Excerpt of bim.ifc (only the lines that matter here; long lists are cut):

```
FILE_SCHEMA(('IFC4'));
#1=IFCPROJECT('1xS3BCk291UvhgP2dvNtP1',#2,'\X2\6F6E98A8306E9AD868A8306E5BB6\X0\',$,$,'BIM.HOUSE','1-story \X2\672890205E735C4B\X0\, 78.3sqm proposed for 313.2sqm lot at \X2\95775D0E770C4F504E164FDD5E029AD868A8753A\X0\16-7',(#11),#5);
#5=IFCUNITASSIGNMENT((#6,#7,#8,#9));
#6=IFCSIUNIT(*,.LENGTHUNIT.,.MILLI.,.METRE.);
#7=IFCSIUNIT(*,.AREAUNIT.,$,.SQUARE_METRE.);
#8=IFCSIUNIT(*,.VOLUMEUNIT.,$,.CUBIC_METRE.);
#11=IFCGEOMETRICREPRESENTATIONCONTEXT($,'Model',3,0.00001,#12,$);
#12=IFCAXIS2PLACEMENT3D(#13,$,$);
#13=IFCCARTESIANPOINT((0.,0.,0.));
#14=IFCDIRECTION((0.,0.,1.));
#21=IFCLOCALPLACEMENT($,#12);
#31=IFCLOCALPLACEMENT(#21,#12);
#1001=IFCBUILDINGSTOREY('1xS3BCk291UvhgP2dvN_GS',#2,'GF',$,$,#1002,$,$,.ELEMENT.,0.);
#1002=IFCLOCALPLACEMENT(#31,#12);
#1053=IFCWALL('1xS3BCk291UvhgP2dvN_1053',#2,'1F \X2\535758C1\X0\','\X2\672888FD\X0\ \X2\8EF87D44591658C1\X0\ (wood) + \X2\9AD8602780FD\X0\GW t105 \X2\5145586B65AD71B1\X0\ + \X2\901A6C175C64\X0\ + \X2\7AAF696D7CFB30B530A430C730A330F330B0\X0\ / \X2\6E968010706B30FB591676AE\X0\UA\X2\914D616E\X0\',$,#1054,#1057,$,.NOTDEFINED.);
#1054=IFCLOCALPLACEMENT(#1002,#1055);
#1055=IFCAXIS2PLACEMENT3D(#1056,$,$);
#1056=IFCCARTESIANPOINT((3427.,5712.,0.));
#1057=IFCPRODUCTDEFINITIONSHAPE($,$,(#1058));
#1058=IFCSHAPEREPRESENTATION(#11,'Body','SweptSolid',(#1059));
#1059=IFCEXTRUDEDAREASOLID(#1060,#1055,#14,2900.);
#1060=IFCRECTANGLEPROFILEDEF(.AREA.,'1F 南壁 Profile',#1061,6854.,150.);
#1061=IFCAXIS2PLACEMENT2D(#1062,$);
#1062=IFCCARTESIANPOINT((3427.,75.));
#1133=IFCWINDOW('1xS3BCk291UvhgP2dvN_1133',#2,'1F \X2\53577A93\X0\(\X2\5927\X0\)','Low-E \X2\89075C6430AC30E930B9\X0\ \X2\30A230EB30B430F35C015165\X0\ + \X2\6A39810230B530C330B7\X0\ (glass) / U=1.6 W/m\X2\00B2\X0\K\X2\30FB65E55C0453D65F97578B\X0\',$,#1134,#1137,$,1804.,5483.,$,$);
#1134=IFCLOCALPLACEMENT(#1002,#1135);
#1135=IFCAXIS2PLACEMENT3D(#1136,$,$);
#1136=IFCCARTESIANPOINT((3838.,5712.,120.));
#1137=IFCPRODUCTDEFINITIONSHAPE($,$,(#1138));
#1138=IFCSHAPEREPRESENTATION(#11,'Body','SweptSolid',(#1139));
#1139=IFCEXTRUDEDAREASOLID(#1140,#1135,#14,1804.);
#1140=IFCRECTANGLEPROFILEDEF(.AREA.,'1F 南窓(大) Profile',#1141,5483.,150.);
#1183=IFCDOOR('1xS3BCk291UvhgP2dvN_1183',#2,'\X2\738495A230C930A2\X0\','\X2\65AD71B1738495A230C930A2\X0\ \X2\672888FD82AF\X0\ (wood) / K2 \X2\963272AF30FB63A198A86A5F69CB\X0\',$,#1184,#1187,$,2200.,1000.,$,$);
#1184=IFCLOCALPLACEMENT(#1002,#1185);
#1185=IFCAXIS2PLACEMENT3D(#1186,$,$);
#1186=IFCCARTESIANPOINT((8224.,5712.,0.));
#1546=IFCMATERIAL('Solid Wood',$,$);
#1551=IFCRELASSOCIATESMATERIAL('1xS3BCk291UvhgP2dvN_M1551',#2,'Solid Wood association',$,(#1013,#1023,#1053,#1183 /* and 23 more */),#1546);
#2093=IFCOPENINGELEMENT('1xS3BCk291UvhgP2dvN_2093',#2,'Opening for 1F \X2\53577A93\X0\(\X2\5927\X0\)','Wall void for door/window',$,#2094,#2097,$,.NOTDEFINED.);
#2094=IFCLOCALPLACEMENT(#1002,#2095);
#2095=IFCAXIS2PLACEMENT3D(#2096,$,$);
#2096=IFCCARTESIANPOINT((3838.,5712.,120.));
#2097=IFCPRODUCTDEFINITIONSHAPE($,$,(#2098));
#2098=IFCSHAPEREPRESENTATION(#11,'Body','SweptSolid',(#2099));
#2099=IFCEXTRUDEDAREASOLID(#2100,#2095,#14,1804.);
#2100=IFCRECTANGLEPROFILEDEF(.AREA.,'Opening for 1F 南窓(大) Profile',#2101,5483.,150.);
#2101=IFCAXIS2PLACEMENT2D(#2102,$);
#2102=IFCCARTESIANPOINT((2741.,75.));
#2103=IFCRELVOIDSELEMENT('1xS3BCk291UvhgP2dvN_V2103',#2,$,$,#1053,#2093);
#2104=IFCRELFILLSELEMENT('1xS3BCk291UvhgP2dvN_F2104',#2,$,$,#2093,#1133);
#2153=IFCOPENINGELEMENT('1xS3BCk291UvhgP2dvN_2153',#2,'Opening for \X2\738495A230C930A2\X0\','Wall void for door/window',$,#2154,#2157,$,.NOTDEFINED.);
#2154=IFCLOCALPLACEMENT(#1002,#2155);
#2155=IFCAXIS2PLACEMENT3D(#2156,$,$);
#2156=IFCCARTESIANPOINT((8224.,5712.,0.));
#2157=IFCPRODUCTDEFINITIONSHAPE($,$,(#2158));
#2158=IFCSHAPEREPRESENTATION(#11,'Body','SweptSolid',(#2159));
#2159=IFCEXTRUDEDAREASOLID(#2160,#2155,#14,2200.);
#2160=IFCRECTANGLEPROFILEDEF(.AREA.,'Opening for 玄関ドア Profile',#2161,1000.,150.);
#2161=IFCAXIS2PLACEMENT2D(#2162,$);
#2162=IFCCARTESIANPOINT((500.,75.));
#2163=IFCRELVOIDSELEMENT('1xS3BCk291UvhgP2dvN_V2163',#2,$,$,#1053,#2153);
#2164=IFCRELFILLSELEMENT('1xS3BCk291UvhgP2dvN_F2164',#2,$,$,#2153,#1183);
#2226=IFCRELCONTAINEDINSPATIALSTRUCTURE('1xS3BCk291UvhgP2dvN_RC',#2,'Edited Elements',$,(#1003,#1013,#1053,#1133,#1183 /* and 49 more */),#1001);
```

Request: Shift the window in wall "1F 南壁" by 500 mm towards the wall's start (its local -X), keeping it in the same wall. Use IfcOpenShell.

```python
import ifcopenshell
import ifcopenshell.api.geometry
import ifcopenshell.util.placement

model = ifcopenshell.open("bim.ifc")

window = model.by_guid("1xS3BCk291UvhgP2dvN_1133")
opening = window.FillsVoids[0].RelatingOpeningElement
wall = opening.VoidsElements[0].RelatingBuildingElement

wall_matrix = ifcopenshell.util.placement.get_local_placement(wall.ObjectPlacement)
shift = wall_matrix[:3, 0] * -500.0
before = ifcopenshell.util.placement.get_local_placement(window.ObjectPlacement)[:3, 3].copy()

# The window is not placed relative to its opening, so move both.
for product in (opening, window):
    matrix = ifcopenshell.util.placement.get_local_placement(product.ObjectPlacement)
    matrix[:3, 3] += shift
    ifcopenshell.api.geometry.edit_object_placement(model, product=product, matrix=matrix, is_si=False)

after = ifcopenshell.util.placement.get_local_placement(window.ObjectPlacement)[:3, 3]
print("window moved by", (after - before).round(3) + 0.0)

model.write("bim_edited.ifc")
```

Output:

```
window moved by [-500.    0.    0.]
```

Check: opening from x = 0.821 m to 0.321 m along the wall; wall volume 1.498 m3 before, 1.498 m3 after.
